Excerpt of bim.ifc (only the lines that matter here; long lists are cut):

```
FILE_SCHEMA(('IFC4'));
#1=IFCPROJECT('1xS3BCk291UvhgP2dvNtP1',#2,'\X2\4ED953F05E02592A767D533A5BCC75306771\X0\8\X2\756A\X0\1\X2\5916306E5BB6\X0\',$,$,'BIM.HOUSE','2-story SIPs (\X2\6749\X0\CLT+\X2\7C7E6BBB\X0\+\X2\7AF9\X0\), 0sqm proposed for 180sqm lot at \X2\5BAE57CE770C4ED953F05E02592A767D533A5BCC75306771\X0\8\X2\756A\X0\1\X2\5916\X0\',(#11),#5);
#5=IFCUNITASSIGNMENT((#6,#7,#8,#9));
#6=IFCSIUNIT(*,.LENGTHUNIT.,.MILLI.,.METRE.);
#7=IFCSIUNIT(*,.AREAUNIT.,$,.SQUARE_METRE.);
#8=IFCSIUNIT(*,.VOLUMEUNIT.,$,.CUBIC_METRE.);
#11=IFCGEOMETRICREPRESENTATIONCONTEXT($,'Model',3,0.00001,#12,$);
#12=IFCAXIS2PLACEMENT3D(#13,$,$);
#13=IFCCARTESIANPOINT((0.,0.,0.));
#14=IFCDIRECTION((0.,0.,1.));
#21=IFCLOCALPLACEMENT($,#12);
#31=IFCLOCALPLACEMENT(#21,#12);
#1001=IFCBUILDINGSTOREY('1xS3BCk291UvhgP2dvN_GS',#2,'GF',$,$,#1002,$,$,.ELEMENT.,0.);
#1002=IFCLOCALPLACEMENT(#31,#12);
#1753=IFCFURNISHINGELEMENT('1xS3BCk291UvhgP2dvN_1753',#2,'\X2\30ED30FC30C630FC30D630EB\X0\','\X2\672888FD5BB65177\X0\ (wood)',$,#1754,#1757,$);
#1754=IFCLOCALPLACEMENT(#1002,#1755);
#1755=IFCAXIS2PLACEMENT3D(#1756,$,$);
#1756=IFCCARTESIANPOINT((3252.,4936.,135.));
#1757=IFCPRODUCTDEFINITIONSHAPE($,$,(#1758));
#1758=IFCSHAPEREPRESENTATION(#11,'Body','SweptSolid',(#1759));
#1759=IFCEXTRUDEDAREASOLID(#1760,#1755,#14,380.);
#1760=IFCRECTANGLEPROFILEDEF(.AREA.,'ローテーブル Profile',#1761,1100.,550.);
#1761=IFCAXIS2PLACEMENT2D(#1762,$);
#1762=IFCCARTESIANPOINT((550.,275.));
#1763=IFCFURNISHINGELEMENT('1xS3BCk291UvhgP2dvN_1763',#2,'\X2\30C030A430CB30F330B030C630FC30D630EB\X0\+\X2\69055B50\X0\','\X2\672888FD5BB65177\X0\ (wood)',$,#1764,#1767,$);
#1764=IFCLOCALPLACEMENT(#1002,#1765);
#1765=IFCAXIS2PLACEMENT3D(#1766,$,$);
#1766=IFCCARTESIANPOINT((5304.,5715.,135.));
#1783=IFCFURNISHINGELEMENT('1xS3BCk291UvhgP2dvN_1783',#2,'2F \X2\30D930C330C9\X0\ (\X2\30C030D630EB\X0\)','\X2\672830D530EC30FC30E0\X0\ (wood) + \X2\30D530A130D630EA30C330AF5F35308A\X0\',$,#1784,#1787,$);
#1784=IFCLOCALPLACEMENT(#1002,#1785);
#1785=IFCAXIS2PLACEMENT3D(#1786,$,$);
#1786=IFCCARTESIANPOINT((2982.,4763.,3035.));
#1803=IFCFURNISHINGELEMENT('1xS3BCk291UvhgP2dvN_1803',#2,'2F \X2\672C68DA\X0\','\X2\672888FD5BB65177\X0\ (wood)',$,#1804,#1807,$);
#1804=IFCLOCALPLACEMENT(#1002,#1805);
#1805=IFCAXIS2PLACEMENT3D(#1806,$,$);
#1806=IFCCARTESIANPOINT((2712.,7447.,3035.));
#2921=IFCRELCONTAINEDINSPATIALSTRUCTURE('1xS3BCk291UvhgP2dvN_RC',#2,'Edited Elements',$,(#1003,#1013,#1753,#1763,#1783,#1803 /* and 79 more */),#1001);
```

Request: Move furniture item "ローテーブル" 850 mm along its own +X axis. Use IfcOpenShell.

```python
import ifcopenshell
import ifcopenshell.api.geometry
import ifcopenshell.util.placement

model = ifcopenshell.open("bim.ifc")

item = model.by_guid("1xS3BCk291UvhgP2dvN_1753")
matrix = ifcopenshell.util.placement.get_local_placement(item.ObjectPlacement)
matrix[:3, 3] += matrix[:3, 0] * 850.0
ifcopenshell.api.geometry.edit_object_placement(model, product=item, matrix=matrix, is_si=False)

print(ifcopenshell.util.placement.get_local_placement(item.ObjectPlacement).round(3) + 0.0)

model.write("bim_edited.ifc")
```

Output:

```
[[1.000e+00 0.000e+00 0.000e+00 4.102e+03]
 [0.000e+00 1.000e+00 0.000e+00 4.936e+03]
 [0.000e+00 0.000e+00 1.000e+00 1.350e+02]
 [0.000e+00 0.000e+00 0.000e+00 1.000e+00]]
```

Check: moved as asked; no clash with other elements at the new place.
